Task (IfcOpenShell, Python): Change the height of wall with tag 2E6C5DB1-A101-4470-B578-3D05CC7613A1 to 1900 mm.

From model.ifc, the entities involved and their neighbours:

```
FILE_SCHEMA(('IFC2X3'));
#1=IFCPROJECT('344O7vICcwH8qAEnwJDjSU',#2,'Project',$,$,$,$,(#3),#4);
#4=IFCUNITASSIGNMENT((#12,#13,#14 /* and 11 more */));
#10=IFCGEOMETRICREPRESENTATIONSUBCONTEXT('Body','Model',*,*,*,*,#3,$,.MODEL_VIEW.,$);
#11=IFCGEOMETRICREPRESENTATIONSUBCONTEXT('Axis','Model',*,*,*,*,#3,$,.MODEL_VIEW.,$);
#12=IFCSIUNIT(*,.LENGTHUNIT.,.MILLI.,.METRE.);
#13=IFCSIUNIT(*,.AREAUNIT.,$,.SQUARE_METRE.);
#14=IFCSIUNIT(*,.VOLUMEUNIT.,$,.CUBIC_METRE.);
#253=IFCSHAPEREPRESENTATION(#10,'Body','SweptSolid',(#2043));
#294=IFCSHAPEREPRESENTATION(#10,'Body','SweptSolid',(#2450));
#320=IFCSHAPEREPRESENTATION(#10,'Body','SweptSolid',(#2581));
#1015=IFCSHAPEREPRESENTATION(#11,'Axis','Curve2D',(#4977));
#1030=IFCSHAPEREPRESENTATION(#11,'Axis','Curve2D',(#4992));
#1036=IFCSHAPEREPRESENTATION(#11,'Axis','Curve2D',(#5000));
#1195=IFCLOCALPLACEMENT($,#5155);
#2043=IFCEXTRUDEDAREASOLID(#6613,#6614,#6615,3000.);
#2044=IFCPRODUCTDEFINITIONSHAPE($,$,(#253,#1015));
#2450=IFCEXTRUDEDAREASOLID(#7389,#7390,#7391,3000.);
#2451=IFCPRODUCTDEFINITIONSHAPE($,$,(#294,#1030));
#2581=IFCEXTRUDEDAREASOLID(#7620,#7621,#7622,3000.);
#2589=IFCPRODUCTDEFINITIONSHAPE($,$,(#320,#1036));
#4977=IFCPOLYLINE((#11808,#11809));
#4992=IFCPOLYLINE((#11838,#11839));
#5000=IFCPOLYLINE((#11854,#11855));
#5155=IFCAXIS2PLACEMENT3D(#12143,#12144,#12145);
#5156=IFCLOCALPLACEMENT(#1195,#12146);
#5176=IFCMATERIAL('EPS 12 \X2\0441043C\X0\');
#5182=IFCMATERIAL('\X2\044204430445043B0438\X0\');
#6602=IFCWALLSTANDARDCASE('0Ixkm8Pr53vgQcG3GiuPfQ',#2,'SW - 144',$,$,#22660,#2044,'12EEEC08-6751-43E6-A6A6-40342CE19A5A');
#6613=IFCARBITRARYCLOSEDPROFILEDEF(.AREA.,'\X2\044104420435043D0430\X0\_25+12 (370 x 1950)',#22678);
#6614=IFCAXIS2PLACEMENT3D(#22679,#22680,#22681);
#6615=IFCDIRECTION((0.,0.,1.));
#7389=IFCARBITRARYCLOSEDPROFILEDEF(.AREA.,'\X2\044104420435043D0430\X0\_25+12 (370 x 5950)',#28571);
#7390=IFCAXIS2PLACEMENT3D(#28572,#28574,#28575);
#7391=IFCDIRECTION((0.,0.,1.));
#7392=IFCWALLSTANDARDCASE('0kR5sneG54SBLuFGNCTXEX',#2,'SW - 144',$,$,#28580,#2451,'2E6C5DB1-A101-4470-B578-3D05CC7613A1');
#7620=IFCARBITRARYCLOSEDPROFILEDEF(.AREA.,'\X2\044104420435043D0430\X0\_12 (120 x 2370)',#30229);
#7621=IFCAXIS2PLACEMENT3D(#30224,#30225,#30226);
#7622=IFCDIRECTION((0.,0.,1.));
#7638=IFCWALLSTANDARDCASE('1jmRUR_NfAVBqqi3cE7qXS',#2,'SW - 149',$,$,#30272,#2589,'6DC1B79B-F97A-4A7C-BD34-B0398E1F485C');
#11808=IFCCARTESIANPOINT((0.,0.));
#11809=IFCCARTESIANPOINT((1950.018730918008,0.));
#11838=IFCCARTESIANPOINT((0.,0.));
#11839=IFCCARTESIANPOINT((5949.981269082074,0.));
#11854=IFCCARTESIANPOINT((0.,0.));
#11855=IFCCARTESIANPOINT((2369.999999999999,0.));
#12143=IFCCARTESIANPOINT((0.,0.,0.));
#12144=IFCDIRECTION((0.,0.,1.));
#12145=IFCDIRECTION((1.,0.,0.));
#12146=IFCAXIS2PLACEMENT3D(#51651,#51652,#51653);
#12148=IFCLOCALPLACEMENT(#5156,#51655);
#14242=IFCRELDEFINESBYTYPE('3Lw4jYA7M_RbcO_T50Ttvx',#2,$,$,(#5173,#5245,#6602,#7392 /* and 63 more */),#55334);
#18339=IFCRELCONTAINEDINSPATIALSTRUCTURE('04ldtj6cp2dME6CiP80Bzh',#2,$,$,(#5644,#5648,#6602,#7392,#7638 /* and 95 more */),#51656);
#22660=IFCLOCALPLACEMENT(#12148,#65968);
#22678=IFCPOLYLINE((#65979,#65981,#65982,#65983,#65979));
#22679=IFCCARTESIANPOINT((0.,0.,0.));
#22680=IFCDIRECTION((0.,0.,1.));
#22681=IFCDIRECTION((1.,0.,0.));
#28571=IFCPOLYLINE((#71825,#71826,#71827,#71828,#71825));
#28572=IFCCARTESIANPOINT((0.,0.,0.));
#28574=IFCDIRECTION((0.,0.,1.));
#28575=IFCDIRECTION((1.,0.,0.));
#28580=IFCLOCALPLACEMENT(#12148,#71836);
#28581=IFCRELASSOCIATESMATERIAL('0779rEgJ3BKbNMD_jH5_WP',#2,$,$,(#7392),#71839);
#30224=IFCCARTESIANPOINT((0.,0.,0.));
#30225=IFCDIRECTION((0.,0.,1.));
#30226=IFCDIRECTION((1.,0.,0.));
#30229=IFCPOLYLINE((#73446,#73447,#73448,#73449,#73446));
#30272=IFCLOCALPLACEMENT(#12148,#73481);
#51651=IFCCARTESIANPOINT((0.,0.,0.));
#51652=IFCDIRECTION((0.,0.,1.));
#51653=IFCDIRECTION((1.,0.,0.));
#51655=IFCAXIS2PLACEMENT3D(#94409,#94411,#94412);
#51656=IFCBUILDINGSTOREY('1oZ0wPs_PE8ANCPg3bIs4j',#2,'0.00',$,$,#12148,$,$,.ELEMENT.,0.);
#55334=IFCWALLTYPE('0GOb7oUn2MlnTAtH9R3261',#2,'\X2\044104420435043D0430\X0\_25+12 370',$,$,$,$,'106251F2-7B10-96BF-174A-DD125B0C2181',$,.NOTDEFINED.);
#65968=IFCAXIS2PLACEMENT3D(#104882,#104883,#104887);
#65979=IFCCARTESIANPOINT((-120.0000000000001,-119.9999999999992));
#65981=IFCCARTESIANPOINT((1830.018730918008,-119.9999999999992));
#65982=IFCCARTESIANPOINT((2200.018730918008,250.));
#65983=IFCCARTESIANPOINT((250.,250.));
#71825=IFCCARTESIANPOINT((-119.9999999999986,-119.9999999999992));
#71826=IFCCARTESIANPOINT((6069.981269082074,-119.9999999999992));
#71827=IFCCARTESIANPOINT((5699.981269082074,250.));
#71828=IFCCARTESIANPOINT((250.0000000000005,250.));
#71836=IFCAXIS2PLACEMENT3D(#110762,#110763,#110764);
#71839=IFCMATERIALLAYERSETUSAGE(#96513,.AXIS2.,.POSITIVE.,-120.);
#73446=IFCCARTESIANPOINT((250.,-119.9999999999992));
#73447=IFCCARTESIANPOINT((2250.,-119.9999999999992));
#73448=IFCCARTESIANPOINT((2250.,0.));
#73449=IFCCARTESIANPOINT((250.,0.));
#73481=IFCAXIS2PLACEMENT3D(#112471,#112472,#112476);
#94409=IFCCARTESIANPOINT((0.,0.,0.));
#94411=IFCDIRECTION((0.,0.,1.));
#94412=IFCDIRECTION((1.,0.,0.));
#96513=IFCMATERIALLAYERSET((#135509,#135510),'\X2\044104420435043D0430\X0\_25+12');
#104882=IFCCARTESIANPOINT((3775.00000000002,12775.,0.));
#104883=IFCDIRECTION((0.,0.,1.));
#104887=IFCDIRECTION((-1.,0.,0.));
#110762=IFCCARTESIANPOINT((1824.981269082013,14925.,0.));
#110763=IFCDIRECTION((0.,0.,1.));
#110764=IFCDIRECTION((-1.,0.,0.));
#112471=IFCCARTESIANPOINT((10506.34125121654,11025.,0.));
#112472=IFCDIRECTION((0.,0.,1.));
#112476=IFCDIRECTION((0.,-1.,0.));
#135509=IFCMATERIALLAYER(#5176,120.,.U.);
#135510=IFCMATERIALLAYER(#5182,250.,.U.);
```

```python
import ifcopenshell
import ifcopenshell.geom
import ifcopenshell.util.representation
import ifcopenshell.util.shape
import ifcopenshell.util.unit

model = ifcopenshell.open("model.ifc")
unit_scale = ifcopenshell.util.unit.calculate_unit_scale(model)
settings = ifcopenshell.geom.settings()


def volume(element):
    """Net volume in cubic metres, openings subtracted."""
    shape = ifcopenshell.geom.create_shape(settings, element)
    return ifcopenshell.util.shape.get_volume(shape.geometry)


wall = model.by_id(7392)
before = volume(wall)

body = ifcopenshell.util.representation.get_representation(wall, "Model", "Body")
solid = body.Items[0]
old_height = solid.Depth
solid.Depth = 1.9 / unit_scale
after = volume(wall)

print(f"height {old_height:g} -> {solid.Depth:g}, volume {before:.3f} -> {after:.3f} m3")

model.write("model_v2.ifc")
```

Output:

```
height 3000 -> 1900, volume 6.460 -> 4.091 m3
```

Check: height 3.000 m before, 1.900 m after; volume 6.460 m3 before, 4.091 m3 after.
